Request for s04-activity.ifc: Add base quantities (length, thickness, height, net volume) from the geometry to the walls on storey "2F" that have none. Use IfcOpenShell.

First a look at what the model holds.

```python
import ifcopenshell
import ifcopenshell.util.element
import ifcopenshell.util.unit

model = ifcopenshell.open("s04-activity.ifc")
print(model.schema)
for unit_type in ("LENGTHUNIT", "AREAUNIT", "VOLUMEUNIT"):
    print(unit_type, ifcopenshell.util.unit.calculate_unit_scale(model, unit_type))
storey = next(s for s in model.by_type("IfcBuildingStorey") if s.Name == "2F")
walls = [e for e in ifcopenshell.util.element.get_decomposition(storey) if e.is_a("IfcWall")]
for e in sorted(walls, key=lambda e: e.id()):
    print(e.id(), e.is_a(), e.Name, list(ifcopenshell.util.element.get_psets(e, qtos_only=True)), sep=" | ")
```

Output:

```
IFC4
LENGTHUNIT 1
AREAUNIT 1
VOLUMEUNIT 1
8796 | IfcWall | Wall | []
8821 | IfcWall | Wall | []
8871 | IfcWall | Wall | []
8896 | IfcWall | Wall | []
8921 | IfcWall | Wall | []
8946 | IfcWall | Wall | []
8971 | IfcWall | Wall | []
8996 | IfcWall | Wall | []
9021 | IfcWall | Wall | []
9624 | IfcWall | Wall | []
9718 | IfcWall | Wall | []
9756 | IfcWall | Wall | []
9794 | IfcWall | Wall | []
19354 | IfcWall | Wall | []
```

```python
import ifcopenshell
import ifcopenshell.api.pset
import ifcopenshell.geom
import ifcopenshell.util.element
import ifcopenshell.util.shape
import ifcopenshell.util.unit

model = ifcopenshell.open("s04-activity.ifc")
unit_scale = ifcopenshell.util.unit.calculate_unit_scale(model)
volume_scale = ifcopenshell.util.unit.calculate_unit_scale(model, "VOLUMEUNIT")
settings = ifcopenshell.geom.settings()

storey = next(s for s in model.by_type("IfcBuildingStorey") if s.Name == "2F")
walls = [e for e in ifcopenshell.util.element.get_decomposition(storey) if e.is_a("IfcWall")]

for e in sorted(walls, key=lambda e: e.id()):
    if ifcopenshell.util.element.get_psets(e, qtos_only=True, should_inherit=False):
        continue
    # Geometry comes back in metres, in the element's own axes.
    shape = ifcopenshell.geom.create_shape(settings, e)
    values = {
        "Length": ifcopenshell.util.shape.get_x(shape.geometry) / unit_scale,
        "Width": ifcopenshell.util.shape.get_y(shape.geometry) / unit_scale,
        "Height": ifcopenshell.util.shape.get_z(shape.geometry) / unit_scale,
        "NetVolume": ifcopenshell.util.shape.get_volume(shape.geometry) / volume_scale,
    }
    qto = ifcopenshell.api.pset.add_qto(model, product=e, name="Qto_WallBaseQuantities")
    ifcopenshell.api.pset.edit_qto(model, qto=qto, properties=values)
    print(e.id(), {k: round(v, 3) for k, v in values.items()})

model.write("s04-activity_edited.ifc")
```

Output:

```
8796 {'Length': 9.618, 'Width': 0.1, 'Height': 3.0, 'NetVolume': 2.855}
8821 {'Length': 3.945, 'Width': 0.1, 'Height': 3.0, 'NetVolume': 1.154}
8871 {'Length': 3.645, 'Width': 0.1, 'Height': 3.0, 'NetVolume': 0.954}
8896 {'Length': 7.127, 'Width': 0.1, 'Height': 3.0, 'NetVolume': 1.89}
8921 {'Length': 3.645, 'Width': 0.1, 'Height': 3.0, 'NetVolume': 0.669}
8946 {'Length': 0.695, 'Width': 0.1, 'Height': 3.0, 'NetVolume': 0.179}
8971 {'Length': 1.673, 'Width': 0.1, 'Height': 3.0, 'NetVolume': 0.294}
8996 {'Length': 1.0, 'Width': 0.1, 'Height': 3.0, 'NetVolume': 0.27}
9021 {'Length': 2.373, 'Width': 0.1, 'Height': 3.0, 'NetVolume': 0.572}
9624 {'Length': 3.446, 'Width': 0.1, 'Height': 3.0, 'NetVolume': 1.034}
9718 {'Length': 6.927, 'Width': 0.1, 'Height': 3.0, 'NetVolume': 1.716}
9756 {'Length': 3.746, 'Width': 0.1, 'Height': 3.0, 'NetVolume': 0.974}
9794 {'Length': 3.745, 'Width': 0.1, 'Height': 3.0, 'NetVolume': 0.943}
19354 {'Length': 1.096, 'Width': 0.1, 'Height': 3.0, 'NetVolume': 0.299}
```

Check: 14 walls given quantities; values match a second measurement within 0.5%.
